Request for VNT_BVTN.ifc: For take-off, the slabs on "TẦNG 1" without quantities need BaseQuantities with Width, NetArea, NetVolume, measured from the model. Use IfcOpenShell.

First a look at what the model holds.

```python
import ifcopenshell
import ifcopenshell.util.element
import ifcopenshell.util.unit

model = ifcopenshell.open("VNT_BVTN.ifc")
print(model.schema)
for unit_type in ("LENGTHUNIT", "AREAUNIT", "VOLUMEUNIT"):
    print(unit_type, ifcopenshell.util.unit.calculate_unit_scale(model, unit_type))
storey = next(s for s in model.by_type("IfcBuildingStorey") if s.Name == "TẦNG 1")
slabs = [e for e in ifcopenshell.util.element.get_decomposition(storey) if e.is_a("IfcSlab")]
for e in sorted(slabs, key=lambda e: e.id()):
    print(e.id(), e.is_a(), e.Name, list(ifcopenshell.util.element.get_psets(e, qtos_only=True)), sep=" | ")
```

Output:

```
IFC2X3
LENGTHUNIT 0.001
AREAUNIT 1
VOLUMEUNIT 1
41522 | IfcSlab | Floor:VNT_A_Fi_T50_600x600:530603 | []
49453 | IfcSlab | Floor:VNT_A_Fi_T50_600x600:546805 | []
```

```python
import ifcopenshell
import ifcopenshell.api.pset
import ifcopenshell.geom
import ifcopenshell.util.element
import ifcopenshell.util.shape
import ifcopenshell.util.unit

model = ifcopenshell.open("VNT_BVTN.ifc")
unit_scale = ifcopenshell.util.unit.calculate_unit_scale(model)
area_scale = ifcopenshell.util.unit.calculate_unit_scale(model, "AREAUNIT")
volume_scale = ifcopenshell.util.unit.calculate_unit_scale(model, "VOLUMEUNIT")
settings = ifcopenshell.geom.settings()

storey = next(s for s in model.by_type("IfcBuildingStorey") if s.Name == "TẦNG 1")
slabs = [e for e in ifcopenshell.util.element.get_decomposition(storey) if e.is_a("IfcSlab")]

for e in sorted(slabs, key=lambda e: e.id()):
    if ifcopenshell.util.element.get_psets(e, qtos_only=True, should_inherit=False):
        continue
    # Geometry comes back in metres, in the element's own axes.
    shape = ifcopenshell.geom.create_shape(settings, e)
    values = {
        "Width": ifcopenshell.util.shape.get_z(shape.geometry) / unit_scale,
        "NetArea": ifcopenshell.util.shape.get_footprint_area(shape.geometry) / area_scale,
        "NetVolume": ifcopenshell.util.shape.get_volume(shape.geometry) / volume_scale,
    }
    qto = ifcopenshell.api.pset.add_qto(model, product=e, name="BaseQuantities")
    ifcopenshell.api.pset.edit_qto(model, qto=qto, properties=values)
    print(e.id(), {k: round(v, 3) for k, v in values.items()})

model.write("VNT_BVTN_rev.ifc")
```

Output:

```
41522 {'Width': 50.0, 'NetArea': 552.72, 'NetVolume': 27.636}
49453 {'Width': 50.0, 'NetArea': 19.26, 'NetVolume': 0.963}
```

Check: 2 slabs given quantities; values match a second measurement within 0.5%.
